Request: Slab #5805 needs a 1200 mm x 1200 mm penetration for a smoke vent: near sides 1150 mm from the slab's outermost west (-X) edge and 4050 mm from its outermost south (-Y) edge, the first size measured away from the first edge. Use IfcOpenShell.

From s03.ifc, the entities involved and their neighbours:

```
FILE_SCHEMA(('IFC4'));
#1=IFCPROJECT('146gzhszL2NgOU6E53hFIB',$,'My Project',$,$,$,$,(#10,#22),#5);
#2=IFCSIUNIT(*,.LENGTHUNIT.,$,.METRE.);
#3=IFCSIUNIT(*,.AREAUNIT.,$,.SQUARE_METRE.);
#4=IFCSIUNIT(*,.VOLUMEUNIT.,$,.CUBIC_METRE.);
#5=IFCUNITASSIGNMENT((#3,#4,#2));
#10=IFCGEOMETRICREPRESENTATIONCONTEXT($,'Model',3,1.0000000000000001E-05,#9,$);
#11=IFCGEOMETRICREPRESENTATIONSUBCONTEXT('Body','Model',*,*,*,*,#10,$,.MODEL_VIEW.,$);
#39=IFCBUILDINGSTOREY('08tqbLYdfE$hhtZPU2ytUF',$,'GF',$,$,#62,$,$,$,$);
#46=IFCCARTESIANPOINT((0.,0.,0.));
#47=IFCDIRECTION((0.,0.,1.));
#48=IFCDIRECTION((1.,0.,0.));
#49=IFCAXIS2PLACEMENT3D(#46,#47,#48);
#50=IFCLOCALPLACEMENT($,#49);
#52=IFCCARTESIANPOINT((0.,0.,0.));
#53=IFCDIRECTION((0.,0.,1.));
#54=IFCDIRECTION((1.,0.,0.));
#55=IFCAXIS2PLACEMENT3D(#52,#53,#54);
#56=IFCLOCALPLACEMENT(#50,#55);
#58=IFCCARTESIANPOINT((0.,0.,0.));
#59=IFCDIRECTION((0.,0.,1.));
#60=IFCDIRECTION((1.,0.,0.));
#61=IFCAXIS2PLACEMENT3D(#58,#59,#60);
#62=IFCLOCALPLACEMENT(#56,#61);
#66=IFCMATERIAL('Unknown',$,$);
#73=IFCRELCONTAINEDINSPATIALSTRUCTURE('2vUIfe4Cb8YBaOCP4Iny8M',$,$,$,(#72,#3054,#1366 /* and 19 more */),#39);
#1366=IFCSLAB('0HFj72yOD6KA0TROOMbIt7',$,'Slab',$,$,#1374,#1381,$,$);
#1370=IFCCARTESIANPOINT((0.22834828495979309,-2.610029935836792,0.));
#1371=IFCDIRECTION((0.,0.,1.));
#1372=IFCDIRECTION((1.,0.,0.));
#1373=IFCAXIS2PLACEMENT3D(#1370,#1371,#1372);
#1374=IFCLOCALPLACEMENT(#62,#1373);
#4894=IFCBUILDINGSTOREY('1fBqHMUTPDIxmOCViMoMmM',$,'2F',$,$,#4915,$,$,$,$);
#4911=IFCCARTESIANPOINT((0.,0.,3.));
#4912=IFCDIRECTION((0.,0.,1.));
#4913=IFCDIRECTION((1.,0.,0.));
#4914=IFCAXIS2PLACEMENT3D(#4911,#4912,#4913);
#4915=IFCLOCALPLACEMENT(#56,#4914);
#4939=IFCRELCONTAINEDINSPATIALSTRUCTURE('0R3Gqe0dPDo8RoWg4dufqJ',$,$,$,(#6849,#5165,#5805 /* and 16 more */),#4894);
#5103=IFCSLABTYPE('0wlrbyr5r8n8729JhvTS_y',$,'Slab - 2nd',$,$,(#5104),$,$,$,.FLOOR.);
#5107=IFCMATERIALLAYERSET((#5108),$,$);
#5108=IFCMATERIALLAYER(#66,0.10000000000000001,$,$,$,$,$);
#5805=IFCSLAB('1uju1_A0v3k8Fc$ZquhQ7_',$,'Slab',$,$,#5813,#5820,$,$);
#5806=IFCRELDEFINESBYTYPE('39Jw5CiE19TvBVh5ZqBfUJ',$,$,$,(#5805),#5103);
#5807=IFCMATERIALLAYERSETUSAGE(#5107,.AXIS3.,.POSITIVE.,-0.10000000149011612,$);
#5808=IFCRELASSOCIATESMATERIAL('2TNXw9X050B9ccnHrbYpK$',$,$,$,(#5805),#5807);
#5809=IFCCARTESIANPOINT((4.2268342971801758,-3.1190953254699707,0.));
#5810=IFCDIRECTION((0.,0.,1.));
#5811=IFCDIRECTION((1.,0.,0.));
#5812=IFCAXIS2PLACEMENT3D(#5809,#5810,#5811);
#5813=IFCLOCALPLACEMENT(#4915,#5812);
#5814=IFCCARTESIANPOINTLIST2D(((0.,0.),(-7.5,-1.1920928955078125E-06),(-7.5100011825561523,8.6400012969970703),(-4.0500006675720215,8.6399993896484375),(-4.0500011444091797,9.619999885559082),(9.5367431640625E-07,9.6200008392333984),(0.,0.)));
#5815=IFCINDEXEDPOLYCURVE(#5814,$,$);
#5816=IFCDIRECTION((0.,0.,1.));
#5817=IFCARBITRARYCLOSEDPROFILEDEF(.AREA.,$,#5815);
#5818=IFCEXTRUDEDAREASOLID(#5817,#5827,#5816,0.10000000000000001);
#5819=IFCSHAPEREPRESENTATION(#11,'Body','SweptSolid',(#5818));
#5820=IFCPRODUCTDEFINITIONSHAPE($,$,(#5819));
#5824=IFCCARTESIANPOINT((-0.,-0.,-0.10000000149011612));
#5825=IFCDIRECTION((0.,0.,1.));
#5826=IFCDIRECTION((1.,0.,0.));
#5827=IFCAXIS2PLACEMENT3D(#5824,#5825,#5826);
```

```python
import numpy as np
import ifcopenshell
import ifcopenshell.api.feature
import ifcopenshell.api.geometry
import ifcopenshell.api.root
import ifcopenshell.geom
import ifcopenshell.util.placement
import ifcopenshell.util.representation
import ifcopenshell.util.shape
import ifcopenshell.util.unit

model = ifcopenshell.open("s03.ifc")
unit_scale = ifcopenshell.util.unit.calculate_unit_scale(model)
settings = ifcopenshell.geom.settings()


def volume(element):
    """Net volume in cubic metres, openings subtracted."""
    shape = ifcopenshell.geom.create_shape(settings, element)
    return ifcopenshell.util.shape.get_volume(shape.geometry)


slab = model.by_guid("1uju1_A0v3k8Fc$ZquhQ7_")
before = volume(slab)

# Extent in the slab's own axes, in metres. The edges named are its -X and -Y sides.
slab_shape = ifcopenshell.geom.create_shape(settings, slab)
vertices = ifcopenshell.util.shape.get_vertices(slab_shape.geometry)
x_min, y_min, bottom = vertices.min(axis=0)
top = vertices[:, 2].max()

opening = ifcopenshell.api.root.create_entity(model, ifc_class="IfcOpeningElement", name="Smoke vent opening", predefined_type="OPENING")
context = ifcopenshell.util.representation.get_context(model, "Model", "Body", "MODEL_VIEW")
width, depth = 1.2, 1.2
outline = [(0.0, 0.0), (width, 0.0), (width, depth), (0.0, depth), (0.0, 0.0)]
# Overshoot both faces by 50 mm so the cut is clean.
shape = ifcopenshell.api.geometry.add_slab_representation(
    model, context=context, depth=top - bottom + 0.1, polyline=outline
)
ifcopenshell.api.geometry.assign_representation(model, product=opening, representation=shape)

matrix = ifcopenshell.util.placement.get_local_placement(slab.ObjectPlacement)
matrix[:, 3] = matrix @ np.append(np.array([x_min + 1.15, y_min + 4.05, bottom - 0.05]) / unit_scale, 1.0)
ifcopenshell.api.geometry.edit_object_placement(model, product=opening, matrix=matrix, is_si=False)
ifcopenshell.api.feature.add_feature(model, feature=opening, element=slab)

after = volume(slab)

print(f"slab volume {before:.3f} -> {after:.3f} m3")

model.write("s03_v2.ifc")
```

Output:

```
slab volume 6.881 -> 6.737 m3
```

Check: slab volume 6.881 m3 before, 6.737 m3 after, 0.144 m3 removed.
